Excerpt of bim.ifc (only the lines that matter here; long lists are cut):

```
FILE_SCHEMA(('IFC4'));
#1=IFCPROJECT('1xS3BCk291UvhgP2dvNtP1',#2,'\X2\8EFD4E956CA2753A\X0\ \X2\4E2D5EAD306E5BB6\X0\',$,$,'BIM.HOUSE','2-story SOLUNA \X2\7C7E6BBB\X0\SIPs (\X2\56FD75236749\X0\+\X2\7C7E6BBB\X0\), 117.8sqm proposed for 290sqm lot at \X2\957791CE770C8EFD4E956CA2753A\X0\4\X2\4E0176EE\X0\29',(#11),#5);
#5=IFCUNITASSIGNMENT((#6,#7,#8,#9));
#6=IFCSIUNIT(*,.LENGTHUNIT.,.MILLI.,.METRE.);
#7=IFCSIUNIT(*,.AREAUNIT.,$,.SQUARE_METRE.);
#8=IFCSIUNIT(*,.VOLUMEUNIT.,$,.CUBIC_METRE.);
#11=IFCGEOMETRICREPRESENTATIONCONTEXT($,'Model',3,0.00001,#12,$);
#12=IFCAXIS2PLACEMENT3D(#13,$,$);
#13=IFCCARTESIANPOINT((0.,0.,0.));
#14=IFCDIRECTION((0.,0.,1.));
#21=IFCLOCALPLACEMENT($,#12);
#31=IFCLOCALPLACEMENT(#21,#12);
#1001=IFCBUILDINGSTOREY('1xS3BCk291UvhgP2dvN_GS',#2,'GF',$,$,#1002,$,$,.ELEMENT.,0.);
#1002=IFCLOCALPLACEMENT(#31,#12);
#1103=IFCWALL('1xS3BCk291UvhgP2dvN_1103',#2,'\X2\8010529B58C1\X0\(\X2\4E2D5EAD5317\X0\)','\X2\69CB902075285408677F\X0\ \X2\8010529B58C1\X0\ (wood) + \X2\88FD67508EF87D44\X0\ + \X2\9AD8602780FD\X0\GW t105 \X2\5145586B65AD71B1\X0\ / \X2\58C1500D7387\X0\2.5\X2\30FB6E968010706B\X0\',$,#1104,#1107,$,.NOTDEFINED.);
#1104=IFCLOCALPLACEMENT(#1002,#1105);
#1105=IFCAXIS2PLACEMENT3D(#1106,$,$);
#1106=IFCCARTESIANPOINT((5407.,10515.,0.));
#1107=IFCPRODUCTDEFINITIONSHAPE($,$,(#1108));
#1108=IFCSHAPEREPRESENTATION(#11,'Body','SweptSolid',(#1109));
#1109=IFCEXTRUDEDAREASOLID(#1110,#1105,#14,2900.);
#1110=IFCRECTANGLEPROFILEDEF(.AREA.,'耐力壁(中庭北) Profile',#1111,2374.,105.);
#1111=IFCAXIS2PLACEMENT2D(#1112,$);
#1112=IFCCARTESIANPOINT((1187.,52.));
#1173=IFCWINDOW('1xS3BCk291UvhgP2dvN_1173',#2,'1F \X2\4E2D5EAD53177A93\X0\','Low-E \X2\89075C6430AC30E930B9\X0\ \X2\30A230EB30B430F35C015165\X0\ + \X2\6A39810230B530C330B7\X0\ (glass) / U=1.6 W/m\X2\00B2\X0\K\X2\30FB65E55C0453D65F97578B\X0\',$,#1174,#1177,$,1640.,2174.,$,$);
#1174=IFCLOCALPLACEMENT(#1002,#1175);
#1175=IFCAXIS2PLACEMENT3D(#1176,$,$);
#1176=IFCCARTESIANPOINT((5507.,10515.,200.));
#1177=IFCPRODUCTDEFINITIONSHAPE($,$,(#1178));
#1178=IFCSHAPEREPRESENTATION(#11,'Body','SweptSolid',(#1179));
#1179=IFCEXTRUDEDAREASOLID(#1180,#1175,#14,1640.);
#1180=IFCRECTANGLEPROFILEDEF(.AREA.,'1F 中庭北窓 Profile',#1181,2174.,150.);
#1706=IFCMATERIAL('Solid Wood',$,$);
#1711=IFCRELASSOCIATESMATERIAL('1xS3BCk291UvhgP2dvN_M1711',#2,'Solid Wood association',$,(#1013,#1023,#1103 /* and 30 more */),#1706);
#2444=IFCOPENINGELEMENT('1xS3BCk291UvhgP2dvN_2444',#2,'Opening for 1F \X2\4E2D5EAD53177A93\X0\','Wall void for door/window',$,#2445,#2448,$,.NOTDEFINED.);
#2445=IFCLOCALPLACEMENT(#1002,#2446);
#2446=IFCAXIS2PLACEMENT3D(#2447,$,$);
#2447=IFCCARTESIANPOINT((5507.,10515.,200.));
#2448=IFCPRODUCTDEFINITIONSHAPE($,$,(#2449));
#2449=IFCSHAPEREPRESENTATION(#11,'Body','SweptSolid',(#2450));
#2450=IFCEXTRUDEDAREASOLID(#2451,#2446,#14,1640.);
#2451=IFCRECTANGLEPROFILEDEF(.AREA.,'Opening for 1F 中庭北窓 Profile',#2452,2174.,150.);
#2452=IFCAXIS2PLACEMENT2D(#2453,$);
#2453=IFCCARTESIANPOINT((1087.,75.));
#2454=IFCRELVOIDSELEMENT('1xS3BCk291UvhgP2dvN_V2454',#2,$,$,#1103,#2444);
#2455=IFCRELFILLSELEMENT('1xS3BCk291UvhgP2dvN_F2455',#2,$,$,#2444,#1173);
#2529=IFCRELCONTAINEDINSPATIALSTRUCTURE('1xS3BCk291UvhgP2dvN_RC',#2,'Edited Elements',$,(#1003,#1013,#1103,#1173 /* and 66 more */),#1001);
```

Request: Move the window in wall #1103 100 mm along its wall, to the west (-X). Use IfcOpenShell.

```python
import ifcopenshell
import ifcopenshell.api.geometry
import ifcopenshell.util.placement
import ifcopenshell.util.unit

model = ifcopenshell.open("bim.ifc")
unit_scale = ifcopenshell.util.unit.calculate_unit_scale(model)

window = model.by_guid("1xS3BCk291UvhgP2dvN_1173")
opening = window.FillsVoids[0].RelatingOpeningElement
wall = opening.VoidsElements[0].RelatingBuildingElement

wall_matrix = ifcopenshell.util.placement.get_local_placement(wall.ObjectPlacement)
shift = wall_matrix[:3, 0] * -0.1 / unit_scale
before = ifcopenshell.util.placement.get_local_placement(window.ObjectPlacement)[:3, 3].copy()

# The window is not placed relative to its opening, so move both.
for product in (opening, window):
    matrix = ifcopenshell.util.placement.get_local_placement(product.ObjectPlacement)
    matrix[:3, 3] += shift
    ifcopenshell.api.geometry.edit_object_placement(model, product=product, matrix=matrix, is_si=False)

after = ifcopenshell.util.placement.get_local_placement(window.ObjectPlacement)[:3, 3]
print("window moved by", (after - before).round(3) + 0.0)

model.write("bim-out.ifc")
```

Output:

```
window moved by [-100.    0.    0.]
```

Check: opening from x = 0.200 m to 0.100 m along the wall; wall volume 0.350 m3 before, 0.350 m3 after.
